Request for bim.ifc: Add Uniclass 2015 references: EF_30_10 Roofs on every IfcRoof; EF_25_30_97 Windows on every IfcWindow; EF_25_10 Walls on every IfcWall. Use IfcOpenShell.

First a look at what the model holds.

```python
import ifcopenshell

model = ifcopenshell.open("bim.ifc")
print(model.schema)
print("classifications:", [c.Name for c in model.by_type("IfcClassification")])
for ifc_class in ("IfcDoor", "IfcRoof", "IfcStair", "IfcWall", "IfcWindow"):
    print(ifc_class, len(model.by_type(ifc_class)))
```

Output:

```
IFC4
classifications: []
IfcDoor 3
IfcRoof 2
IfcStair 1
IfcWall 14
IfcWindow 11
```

```python
import ifcopenshell
import ifcopenshell.api.classification

model = ifcopenshell.open("bim.ifc")

system = ifcopenshell.api.classification.add_classification(model, classification="Uniclass 2015")

codes = {
    "IfcRoof": ("EF_30_10", "Roofs"),
    "IfcWindow": ("EF_25_30_97", "Windows"),
    "IfcWall": ("EF_25_10", "Walls"),
}
for ifc_class, (code, name) in codes.items():
    products = model.by_type(ifc_class)
    ifcopenshell.api.classification.add_reference(
        model, products=products, classification=system, identification=code, name=name
    )
    print(code, len(products))

model.write("bim_updated.ifc")
```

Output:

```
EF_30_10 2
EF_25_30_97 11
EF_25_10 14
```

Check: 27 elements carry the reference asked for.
